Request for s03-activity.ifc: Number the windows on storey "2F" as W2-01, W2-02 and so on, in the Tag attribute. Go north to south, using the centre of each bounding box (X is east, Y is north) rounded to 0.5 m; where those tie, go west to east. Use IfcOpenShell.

First a look at what the model holds.

```python
import ifcopenshell
import ifcopenshell.util.element
import ifcopenshell.util.placement

model = ifcopenshell.open("s03-activity.ifc")
print(model.schema)
storey = next(s for s in model.by_type("IfcBuildingStorey") if s.Name == "2F")
windows = [e for e in ifcopenshell.util.element.get_decomposition(storey) if e.is_a("IfcWindow")]
for e in sorted(windows, key=lambda e: e.id()):
    origin = ifcopenshell.util.placement.get_local_placement(e.ObjectPlacement)[:3, 3]
    print(e.id(), e.Tag, e.Name, origin.round(2) + 0.0, sep=" | ")
```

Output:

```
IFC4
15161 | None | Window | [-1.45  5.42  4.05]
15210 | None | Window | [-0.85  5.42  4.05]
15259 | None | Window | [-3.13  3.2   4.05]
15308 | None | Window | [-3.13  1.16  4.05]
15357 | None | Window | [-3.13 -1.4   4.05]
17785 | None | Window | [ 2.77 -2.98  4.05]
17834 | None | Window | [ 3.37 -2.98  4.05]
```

```python
import ifcopenshell
import ifcopenshell.geom
import ifcopenshell.util.element
import ifcopenshell.util.shape

model = ifcopenshell.open("s03-activity.ifc")
settings = ifcopenshell.geom.settings()
settings.set("use-world-coords", True)


def centre(element):
    shape = ifcopenshell.geom.create_shape(settings, element)
    return ifcopenshell.util.shape.get_bbox_centroid(shape.geometry)


storey = next(s for s in model.by_type("IfcBuildingStorey") if s.Name == "2F")
windows = [e for e in ifcopenshell.util.element.get_decomposition(storey) if e.is_a("IfcWindow")]

# Insertion points can sit at a corner or the storey origin, so sort by the geometry (in metres).
centres = {e: centre(e) for e in windows}
windows.sort(key=lambda e: (-round(centres[e][1] / 0.5), centres[e][0]))

for i, e in enumerate(windows, start=1):
    number = f"W2-{i:02d}"
    e.Tag = number
    print(e.id(), number)

model.write("s03-activity_rev.ifc")
```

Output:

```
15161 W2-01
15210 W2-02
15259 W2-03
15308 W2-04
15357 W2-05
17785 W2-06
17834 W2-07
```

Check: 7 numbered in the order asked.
